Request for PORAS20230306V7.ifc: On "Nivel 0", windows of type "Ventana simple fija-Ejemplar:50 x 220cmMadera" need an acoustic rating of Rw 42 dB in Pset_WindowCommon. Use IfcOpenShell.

First a look at what the model holds.

```python
import ifcopenshell
import ifcopenshell.util.element

model = ifcopenshell.open("PORAS20230306V7.ifc")
print(model.schema)
storey = next(s for s in model.by_type("IfcBuildingStorey") if s.Name == "Nivel 0")
windows = [e for e in ifcopenshell.util.element.get_decomposition(storey) if e.is_a("IfcWindow")]
seen = {}
for e in windows:
    element_type = ifcopenshell.util.element.get_type(e)
    key = (element_type.Name if element_type != e and element_type else None, ifcopenshell.util.element.get_pset(e, "Pset_WindowCommon", "AcousticRating"))
    seen[key] = seen.get(key, 0) + 1
for (name, value), count in sorted(seen.items(), key=str):
    print(count, "x", name, "|", value)
```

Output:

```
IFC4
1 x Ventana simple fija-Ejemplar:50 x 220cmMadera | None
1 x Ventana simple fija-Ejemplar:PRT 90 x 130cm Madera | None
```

```python
import ifcopenshell
import ifcopenshell.api.pset
import ifcopenshell.util.element

model = ifcopenshell.open("PORAS20230306V7.ifc")

storey = next(s for s in model.by_type("IfcBuildingStorey") if s.Name == "Nivel 0")
windows = [e for e in ifcopenshell.util.element.get_decomposition(storey) if e.is_a("IfcWindow")]

count = 0
for e in windows:
    element_type = ifcopenshell.util.element.get_type(e)
    if element_type in (None, e) or element_type.Name != "Ventana simple fija-Ejemplar:50 x 220cmMadera":
        continue
    # add_pset returns the element's existing set when there is one.
    pset = ifcopenshell.api.pset.add_pset(model, product=e, name="Pset_WindowCommon")
    ifcopenshell.api.pset.edit_pset(model, pset=pset, properties={"AcousticRating": "Rw 42 dB"})
    count += 1

print(count, "windows updated")

model.write("PORAS20230306V7_edited.ifc")
```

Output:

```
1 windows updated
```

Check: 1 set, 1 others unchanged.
